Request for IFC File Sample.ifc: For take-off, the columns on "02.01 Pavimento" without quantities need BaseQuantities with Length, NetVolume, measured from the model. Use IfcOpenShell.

First a look at what the model holds.

```python
import ifcopenshell
import ifcopenshell.util.element
import ifcopenshell.util.unit

model = ifcopenshell.open("IFC File Sample.ifc")
print(model.schema)
for unit_type in ("LENGTHUNIT", "AREAUNIT", "VOLUMEUNIT"):
    print(unit_type, ifcopenshell.util.unit.calculate_unit_scale(model, unit_type))
storey = next(s for s in model.by_type("IfcBuildingStorey") if s.Name == "02.01 Pavimento")
columns = [e for e in ifcopenshell.util.element.get_decomposition(storey) if e.is_a("IfcColumn")]
for e in sorted(columns, key=lambda e: e.id()):
    print(e.id(), e.is_a(), e.Name, list(ifcopenshell.util.element.get_psets(e, qtos_only=True)), sep=" | ")
```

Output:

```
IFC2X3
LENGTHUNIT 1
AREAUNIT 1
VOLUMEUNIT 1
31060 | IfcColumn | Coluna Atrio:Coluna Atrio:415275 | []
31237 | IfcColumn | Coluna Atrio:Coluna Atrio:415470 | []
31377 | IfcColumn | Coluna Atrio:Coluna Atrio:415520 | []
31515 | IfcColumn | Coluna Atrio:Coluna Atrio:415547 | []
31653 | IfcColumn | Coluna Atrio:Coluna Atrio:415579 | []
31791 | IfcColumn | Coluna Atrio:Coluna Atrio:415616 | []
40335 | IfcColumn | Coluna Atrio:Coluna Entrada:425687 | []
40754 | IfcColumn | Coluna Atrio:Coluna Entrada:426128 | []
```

```python
import ifcopenshell
import ifcopenshell.api.pset
import ifcopenshell.geom
import ifcopenshell.util.element
import ifcopenshell.util.shape
import ifcopenshell.util.unit

model = ifcopenshell.open("IFC File Sample.ifc")
unit_scale = ifcopenshell.util.unit.calculate_unit_scale(model)
volume_scale = ifcopenshell.util.unit.calculate_unit_scale(model, "VOLUMEUNIT")
settings = ifcopenshell.geom.settings()

storey = next(s for s in model.by_type("IfcBuildingStorey") if s.Name == "02.01 Pavimento")
columns = [e for e in ifcopenshell.util.element.get_decomposition(storey) if e.is_a("IfcColumn")]

for e in sorted(columns, key=lambda e: e.id()):
    if ifcopenshell.util.element.get_psets(e, qtos_only=True, should_inherit=False):
        continue
    # Geometry comes back in metres, in the element's own axes.
    shape = ifcopenshell.geom.create_shape(settings, e)
    values = {
        "Length": ifcopenshell.util.shape.get_z(shape.geometry) / unit_scale,
        "NetVolume": ifcopenshell.util.shape.get_volume(shape.geometry) / volume_scale,
    }
    qto = ifcopenshell.api.pset.add_qto(model, product=e, name="BaseQuantities")
    ifcopenshell.api.pset.edit_qto(model, qto=qto, properties=values)
    print(e.id(), {k: round(v, 3) for k, v in values.items()})

model.write("IFC File Sample_updated.ifc")
```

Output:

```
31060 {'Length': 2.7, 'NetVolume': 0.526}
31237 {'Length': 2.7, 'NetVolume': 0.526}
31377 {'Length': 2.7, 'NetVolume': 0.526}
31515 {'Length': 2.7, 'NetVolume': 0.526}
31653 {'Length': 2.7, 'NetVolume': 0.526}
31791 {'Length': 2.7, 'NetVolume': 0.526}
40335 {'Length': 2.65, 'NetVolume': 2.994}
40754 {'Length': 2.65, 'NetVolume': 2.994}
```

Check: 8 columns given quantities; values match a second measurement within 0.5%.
